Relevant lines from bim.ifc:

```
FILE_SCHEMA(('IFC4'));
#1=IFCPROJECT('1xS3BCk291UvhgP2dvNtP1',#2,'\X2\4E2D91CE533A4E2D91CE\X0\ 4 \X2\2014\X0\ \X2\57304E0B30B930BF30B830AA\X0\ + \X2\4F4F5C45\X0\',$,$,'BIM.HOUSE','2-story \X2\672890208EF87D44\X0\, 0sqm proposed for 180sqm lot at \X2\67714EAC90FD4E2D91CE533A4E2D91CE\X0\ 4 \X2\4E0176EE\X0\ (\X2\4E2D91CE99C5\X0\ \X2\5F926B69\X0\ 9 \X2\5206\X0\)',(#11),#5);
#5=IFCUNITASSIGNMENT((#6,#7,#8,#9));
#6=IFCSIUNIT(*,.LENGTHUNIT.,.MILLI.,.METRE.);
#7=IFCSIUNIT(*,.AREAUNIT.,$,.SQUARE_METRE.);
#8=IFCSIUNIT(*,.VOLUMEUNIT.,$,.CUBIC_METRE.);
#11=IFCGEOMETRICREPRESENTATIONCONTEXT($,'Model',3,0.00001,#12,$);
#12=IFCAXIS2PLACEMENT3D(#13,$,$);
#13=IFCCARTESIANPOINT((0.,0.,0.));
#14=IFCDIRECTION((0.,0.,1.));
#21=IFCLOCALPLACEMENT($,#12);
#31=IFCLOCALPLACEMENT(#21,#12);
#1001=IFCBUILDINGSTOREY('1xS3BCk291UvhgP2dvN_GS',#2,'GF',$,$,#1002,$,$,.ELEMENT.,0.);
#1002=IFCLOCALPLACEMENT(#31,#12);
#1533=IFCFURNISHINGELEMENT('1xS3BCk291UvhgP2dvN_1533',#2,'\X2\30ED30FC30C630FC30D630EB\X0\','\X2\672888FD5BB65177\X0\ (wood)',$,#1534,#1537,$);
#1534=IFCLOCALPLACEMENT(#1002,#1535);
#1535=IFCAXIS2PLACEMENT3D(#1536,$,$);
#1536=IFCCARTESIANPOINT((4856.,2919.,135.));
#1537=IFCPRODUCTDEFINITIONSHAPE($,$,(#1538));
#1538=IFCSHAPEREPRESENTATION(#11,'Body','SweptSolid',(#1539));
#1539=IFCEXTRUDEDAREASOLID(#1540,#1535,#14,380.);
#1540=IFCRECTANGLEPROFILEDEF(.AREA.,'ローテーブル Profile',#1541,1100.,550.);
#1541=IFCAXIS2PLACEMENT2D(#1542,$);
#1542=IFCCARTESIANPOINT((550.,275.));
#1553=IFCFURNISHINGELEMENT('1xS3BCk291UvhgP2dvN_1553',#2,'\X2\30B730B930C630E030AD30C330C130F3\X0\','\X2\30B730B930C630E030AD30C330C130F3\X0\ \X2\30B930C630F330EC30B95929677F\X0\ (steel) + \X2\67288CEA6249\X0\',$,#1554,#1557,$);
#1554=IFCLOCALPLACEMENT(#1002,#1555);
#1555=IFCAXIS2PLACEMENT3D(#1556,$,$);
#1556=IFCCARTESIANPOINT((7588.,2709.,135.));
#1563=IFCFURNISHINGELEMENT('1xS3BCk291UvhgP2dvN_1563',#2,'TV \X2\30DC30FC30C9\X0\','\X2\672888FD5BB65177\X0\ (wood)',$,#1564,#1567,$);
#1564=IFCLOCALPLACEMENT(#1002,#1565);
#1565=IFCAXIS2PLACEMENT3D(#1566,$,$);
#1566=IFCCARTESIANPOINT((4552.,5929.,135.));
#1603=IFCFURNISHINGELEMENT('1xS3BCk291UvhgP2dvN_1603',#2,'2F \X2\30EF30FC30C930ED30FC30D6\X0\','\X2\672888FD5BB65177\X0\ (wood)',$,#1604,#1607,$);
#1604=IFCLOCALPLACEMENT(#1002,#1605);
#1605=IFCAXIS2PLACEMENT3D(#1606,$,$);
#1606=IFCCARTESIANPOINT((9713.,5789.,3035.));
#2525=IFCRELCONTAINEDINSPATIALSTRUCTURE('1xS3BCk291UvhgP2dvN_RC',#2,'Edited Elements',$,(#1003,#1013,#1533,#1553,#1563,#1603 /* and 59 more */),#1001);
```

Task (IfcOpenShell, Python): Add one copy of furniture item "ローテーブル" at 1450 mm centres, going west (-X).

```python
import numpy as np
import ifcopenshell
import ifcopenshell.api.geometry
import ifcopenshell.api.root
import ifcopenshell.util.element
import ifcopenshell.util.placement

model = ifcopenshell.open("bim.ifc")


def reuse_history(source, copy):
    """copy_class also copies each property set's owner history, people and application; keep the originals."""
    for rel in copy.IsDefinedBy:
        if rel.is_a("IfcRelDefinesByProperties") and (history := rel.RelatingPropertyDefinition.OwnerHistory):
            rel.RelatingPropertyDefinition.OwnerHistory = source.OwnerHistory
            ifcopenshell.util.element.remove_deep2(model, history)


source = model.by_guid("1xS3BCk291UvhgP2dvN_1533")
base = ifcopenshell.util.placement.get_local_placement(source.ObjectPlacement)
step = np.array([-1.0, 0.0, 0.0]) * 1450.0

for i in range(1, 2):
    copy = ifcopenshell.api.root.copy_class(model, product=source)
    copy.Representation = ifcopenshell.util.element.copy_deep(
        model, source.Representation, exclude=["IfcGeometricRepresentationContext", "IfcRepresentationMap"]
    )
    reuse_history(source, copy)
    matrix = base.copy()
    matrix[:3, 3] += i * step
    print("added at", matrix[:3, 3].round(3) + 0.0)
    ifcopenshell.api.geometry.edit_object_placement(model, product=copy, matrix=matrix, is_si=False)

model.write("bim_updated.ifc")
```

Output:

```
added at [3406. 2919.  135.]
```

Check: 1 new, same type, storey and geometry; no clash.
